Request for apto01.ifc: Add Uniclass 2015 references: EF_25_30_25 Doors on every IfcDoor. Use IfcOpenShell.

First a look at what the model holds.

```python
import ifcopenshell

model = ifcopenshell.open("apto01.ifc")
print(model.schema)
print("classifications:", [c.Name for c in model.by_type("IfcClassification")])
for ifc_class in ("IfcDoor", "IfcRoof", "IfcStair", "IfcWall", "IfcWindow"):
    print(ifc_class, len(model.by_type(ifc_class)))
```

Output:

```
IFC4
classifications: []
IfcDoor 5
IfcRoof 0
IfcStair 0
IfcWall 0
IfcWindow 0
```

```python
import ifcopenshell
import ifcopenshell.api.classification

model = ifcopenshell.open("apto01.ifc")

system = ifcopenshell.api.classification.add_classification(model, classification="Uniclass 2015")

codes = {
    "IfcDoor": ("EF_25_30_25", "Doors"),
}
for ifc_class, (code, name) in codes.items():
    products = model.by_type(ifc_class)
    ifcopenshell.api.classification.add_reference(
        model, products=products, classification=system, identification=code, name=name
    )
    print(code, len(products))

model.write("apto01_v2.ifc")
```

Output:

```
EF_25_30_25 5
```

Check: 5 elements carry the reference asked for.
